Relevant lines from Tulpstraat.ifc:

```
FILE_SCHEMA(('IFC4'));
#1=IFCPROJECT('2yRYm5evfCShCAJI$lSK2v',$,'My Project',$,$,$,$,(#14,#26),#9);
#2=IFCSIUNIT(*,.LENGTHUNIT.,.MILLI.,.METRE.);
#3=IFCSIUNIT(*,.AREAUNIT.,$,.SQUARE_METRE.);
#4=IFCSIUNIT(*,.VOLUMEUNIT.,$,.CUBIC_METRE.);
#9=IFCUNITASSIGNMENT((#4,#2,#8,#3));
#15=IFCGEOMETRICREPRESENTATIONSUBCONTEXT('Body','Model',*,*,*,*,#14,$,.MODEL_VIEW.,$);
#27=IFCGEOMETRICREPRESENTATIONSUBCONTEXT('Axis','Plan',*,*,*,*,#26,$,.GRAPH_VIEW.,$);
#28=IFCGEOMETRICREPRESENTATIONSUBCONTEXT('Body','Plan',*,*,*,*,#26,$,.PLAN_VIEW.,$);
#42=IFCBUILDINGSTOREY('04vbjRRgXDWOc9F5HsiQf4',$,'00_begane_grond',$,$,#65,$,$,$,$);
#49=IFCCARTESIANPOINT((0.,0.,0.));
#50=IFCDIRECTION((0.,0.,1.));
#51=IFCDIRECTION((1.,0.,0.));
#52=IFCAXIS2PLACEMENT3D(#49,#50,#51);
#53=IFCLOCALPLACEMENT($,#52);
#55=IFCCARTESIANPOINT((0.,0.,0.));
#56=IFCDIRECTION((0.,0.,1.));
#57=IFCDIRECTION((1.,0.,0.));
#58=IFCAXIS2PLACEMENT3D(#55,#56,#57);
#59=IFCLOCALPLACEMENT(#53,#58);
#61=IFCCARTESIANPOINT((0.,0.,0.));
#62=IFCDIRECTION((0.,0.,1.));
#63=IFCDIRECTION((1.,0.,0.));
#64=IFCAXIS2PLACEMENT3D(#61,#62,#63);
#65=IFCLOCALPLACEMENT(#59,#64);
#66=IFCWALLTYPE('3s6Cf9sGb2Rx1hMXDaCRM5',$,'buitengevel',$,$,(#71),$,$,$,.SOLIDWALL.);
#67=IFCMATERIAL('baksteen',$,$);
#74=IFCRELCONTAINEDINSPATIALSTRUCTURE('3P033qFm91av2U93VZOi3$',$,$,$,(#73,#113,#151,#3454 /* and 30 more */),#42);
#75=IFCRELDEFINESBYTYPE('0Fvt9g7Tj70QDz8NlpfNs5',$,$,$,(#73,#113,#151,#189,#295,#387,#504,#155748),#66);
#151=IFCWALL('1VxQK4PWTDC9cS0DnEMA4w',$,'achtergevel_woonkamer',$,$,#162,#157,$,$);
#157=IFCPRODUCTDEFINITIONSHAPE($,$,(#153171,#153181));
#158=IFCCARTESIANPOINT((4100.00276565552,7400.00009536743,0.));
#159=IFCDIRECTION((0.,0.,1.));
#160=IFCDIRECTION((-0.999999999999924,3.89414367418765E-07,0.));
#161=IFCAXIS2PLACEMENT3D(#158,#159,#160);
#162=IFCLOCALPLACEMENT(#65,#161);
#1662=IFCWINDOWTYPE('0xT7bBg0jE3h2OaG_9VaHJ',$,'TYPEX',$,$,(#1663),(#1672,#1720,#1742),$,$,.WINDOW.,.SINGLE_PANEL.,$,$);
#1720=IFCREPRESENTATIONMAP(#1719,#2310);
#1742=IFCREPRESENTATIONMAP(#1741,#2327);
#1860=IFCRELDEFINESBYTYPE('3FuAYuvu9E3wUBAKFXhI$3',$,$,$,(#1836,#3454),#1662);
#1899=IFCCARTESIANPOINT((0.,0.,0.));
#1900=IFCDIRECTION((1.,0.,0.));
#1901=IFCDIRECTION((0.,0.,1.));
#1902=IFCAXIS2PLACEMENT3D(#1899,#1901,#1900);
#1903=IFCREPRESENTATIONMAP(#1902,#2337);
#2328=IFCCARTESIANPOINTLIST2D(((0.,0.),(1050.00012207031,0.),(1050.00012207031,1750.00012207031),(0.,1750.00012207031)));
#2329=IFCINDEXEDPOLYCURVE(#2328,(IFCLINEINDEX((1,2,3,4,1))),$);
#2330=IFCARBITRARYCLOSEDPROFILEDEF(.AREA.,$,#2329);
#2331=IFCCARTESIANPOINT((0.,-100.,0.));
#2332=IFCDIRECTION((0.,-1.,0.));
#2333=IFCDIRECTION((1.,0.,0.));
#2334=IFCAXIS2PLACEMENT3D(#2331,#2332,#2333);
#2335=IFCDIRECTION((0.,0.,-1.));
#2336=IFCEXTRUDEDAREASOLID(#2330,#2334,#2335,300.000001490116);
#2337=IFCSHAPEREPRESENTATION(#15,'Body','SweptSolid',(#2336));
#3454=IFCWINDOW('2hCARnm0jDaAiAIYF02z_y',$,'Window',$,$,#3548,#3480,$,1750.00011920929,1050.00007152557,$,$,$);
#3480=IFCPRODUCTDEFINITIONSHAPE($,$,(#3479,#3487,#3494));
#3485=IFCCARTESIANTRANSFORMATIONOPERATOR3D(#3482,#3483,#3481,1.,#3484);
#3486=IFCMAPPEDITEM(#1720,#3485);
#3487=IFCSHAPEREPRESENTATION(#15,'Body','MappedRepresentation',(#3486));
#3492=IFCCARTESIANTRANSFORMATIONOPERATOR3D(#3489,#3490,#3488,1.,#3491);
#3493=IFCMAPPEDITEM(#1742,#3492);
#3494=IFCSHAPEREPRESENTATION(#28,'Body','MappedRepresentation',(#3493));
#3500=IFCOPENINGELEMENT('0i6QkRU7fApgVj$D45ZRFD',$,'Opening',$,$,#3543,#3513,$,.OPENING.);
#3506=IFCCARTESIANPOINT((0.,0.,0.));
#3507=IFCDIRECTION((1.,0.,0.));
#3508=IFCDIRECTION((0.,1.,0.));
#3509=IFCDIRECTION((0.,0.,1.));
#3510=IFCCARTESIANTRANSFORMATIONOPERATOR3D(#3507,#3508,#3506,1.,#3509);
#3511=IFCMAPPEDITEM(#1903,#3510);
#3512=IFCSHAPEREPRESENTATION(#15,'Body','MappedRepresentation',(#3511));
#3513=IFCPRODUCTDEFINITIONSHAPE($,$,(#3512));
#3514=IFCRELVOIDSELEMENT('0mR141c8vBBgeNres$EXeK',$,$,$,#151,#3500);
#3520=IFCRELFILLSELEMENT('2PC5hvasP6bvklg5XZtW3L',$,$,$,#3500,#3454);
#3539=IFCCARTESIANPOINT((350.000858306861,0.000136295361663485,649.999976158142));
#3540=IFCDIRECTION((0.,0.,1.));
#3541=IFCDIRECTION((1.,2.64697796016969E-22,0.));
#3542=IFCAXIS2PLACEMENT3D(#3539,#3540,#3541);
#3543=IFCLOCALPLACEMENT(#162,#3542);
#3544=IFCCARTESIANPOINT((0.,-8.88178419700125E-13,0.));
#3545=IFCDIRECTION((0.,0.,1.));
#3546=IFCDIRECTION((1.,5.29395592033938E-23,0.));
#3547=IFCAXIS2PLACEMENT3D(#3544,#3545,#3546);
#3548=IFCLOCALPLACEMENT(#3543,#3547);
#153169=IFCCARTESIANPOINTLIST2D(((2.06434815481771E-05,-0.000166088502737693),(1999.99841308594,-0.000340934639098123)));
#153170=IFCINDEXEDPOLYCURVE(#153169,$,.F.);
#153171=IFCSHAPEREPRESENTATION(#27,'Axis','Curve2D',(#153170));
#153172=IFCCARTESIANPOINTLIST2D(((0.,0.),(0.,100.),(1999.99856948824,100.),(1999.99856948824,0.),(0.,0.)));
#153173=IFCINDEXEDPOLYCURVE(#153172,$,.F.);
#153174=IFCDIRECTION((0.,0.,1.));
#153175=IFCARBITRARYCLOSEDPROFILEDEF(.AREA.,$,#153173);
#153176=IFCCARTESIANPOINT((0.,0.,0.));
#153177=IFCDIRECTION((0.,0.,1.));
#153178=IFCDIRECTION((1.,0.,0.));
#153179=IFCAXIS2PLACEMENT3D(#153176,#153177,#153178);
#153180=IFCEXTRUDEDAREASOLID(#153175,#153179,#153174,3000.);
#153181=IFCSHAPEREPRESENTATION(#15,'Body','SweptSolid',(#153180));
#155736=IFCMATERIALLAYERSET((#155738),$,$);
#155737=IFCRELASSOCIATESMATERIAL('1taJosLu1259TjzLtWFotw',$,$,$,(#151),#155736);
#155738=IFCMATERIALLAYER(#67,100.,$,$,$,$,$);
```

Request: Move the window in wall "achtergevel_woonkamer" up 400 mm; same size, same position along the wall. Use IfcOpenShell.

```python
import numpy as np
import ifcopenshell
import ifcopenshell.api.geometry
import ifcopenshell.util.placement
import ifcopenshell.util.unit

model = ifcopenshell.open("Tulpstraat.ifc")
unit_scale = ifcopenshell.util.unit.calculate_unit_scale(model)

window = model.by_guid("2hCARnm0jDaAiAIYF02z_y")
opening = window.FillsVoids[0].RelatingOpeningElement
dz = 0.4 / unit_scale

shift = np.array([0.0, 0.0, dz])
# The window is placed relative to its opening, so it follows when the opening moves.
matrix = ifcopenshell.util.placement.get_local_placement(opening.ObjectPlacement)
matrix[:3, 3] += shift
ifcopenshell.api.geometry.edit_object_placement(
    model, product=opening, matrix=matrix, is_si=False, should_transform_children=True
)

print(f"moved by {dz * unit_scale:+.3f} m")

model.write("Tulpstraat_v2.ifc")
```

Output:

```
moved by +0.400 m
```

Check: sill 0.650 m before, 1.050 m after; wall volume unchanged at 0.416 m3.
